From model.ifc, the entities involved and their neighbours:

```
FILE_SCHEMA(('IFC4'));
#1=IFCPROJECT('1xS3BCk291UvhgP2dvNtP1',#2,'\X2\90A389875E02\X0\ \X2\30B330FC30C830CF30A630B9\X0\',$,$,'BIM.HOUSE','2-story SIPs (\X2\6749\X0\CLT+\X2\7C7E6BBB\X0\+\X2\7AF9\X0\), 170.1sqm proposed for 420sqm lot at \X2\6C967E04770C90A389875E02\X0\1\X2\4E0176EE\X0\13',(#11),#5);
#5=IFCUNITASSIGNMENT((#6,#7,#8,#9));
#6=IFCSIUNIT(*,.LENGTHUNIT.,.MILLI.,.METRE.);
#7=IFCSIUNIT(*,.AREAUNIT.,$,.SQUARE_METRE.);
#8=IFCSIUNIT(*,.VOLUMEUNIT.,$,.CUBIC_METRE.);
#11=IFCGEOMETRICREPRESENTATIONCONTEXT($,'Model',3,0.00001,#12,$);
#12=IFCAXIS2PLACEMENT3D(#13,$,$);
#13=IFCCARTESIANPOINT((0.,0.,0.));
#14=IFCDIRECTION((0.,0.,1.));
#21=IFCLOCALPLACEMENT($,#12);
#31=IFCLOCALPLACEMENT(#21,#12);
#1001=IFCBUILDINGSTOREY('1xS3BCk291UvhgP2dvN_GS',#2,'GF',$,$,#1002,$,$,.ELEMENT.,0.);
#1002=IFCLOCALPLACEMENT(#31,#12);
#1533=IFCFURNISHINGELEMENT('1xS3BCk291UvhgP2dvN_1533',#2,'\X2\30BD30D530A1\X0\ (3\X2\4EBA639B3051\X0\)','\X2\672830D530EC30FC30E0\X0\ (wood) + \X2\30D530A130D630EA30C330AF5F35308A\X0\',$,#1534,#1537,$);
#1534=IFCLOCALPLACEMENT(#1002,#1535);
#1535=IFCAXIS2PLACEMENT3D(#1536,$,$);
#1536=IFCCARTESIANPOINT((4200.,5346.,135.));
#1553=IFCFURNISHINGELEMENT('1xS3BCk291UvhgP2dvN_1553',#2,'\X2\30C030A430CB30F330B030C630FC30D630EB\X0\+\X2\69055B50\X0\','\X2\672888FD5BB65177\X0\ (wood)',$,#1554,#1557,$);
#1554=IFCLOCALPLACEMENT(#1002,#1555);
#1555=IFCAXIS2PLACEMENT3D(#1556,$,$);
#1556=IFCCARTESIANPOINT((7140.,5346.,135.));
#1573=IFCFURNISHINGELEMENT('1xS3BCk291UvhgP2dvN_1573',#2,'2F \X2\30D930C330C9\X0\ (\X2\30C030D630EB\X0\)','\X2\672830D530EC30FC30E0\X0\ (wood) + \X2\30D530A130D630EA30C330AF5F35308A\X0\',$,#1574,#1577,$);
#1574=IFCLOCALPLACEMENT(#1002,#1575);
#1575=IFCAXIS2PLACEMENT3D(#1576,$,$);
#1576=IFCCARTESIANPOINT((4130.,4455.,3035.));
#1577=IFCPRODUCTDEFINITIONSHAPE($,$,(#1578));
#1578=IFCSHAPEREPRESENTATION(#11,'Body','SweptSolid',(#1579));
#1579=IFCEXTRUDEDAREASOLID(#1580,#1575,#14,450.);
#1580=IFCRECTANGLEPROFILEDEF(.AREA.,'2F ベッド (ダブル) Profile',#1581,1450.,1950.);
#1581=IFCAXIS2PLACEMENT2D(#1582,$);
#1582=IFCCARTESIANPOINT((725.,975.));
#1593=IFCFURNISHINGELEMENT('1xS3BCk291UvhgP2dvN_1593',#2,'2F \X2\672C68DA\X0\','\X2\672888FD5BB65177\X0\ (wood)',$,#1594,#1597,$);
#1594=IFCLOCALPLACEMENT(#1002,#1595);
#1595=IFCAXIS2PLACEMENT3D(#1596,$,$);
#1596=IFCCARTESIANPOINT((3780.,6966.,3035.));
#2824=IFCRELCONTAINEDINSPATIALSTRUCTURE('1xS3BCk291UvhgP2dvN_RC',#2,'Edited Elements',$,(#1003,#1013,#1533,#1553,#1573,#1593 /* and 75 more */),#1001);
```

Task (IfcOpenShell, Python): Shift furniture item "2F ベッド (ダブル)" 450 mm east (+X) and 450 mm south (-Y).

```python
import ifcopenshell
import ifcopenshell.api.geometry
import ifcopenshell.util.placement

model = ifcopenshell.open("model.ifc")

item = model.by_id(1573)
matrix = ifcopenshell.util.placement.get_local_placement(item.ObjectPlacement)
matrix[0, 3] += 450.0
matrix[1, 3] -= 450.0
ifcopenshell.api.geometry.edit_object_placement(model, product=item, matrix=matrix, is_si=False)

print(ifcopenshell.util.placement.get_local_placement(item.ObjectPlacement).round(3) + 0.0)

model.write("model_edited.ifc")
```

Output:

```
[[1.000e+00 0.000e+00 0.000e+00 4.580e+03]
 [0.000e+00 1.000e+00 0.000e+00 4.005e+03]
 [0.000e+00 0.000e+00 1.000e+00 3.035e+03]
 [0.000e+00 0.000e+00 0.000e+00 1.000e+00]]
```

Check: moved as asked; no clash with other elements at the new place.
